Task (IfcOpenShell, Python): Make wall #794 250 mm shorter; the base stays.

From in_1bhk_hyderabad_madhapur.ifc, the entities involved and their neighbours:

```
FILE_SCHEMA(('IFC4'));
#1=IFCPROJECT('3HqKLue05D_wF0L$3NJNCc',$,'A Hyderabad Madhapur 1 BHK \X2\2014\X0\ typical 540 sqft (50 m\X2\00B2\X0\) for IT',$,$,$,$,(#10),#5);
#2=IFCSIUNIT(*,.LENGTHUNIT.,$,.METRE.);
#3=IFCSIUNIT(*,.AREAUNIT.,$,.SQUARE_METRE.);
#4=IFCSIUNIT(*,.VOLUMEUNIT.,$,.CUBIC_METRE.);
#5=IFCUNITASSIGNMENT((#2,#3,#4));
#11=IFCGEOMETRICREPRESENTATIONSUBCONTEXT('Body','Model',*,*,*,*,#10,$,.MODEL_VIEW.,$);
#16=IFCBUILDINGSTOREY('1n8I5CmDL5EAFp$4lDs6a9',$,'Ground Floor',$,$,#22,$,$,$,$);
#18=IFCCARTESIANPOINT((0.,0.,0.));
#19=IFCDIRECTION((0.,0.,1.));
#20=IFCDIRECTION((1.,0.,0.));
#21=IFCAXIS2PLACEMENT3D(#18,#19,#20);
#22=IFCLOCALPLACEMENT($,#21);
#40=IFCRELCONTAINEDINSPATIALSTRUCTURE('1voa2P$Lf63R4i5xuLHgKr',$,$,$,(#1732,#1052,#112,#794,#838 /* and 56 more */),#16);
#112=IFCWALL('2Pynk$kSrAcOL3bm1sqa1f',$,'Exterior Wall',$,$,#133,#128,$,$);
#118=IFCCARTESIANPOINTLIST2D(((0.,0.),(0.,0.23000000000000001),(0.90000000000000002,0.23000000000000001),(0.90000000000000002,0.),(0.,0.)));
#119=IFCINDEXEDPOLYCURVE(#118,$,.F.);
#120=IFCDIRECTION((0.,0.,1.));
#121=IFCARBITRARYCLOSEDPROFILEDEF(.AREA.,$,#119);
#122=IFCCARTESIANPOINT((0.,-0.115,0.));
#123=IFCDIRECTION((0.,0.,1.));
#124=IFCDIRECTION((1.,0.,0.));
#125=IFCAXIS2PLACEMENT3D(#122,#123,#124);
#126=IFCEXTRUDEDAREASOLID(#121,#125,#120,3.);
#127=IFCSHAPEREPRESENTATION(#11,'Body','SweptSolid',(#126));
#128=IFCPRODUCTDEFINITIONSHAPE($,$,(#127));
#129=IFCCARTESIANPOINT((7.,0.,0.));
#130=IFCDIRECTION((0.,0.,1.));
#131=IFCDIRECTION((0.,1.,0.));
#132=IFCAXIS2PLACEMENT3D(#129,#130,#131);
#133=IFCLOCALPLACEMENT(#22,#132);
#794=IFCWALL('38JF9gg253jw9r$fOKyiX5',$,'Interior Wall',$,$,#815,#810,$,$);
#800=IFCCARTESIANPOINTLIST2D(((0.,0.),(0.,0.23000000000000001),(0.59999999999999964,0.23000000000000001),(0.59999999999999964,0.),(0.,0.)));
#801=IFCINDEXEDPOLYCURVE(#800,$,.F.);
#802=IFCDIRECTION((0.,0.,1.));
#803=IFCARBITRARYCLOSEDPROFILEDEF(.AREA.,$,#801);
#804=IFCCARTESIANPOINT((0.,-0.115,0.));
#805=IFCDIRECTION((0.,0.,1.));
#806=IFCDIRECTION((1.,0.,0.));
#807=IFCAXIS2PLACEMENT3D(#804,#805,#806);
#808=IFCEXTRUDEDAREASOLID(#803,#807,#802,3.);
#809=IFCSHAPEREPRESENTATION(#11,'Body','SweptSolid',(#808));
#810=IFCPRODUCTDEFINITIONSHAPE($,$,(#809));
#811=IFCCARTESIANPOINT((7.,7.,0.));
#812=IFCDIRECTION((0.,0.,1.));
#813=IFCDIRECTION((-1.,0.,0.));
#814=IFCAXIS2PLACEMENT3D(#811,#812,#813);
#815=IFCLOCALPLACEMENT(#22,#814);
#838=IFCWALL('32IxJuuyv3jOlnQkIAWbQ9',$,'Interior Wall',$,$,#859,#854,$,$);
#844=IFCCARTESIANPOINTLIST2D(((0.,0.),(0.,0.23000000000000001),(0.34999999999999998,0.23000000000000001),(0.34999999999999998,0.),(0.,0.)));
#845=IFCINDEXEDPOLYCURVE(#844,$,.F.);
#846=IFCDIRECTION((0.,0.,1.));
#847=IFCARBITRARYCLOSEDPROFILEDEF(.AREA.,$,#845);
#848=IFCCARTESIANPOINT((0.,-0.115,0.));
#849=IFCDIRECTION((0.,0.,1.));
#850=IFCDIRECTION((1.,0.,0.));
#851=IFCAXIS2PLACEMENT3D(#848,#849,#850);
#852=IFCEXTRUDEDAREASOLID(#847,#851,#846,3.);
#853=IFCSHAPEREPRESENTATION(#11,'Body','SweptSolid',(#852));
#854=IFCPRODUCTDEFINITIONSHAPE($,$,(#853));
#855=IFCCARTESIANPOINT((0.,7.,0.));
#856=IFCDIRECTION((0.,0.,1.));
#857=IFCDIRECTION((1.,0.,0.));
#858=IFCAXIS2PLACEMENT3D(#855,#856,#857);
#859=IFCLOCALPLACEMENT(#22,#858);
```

```python
import ifcopenshell
import ifcopenshell.geom
import ifcopenshell.util.representation
import ifcopenshell.util.shape

model = ifcopenshell.open("in_1bhk_hyderabad_madhapur.ifc")
settings = ifcopenshell.geom.settings()


def volume(element):
    """Net volume in cubic metres, openings subtracted."""
    shape = ifcopenshell.geom.create_shape(settings, element)
    return ifcopenshell.util.shape.get_volume(shape.geometry)


wall = model.by_guid("38JF9gg253jw9r$fOKyiX5")
before = volume(wall)

body = ifcopenshell.util.representation.get_representation(wall, "Model", "Body")
solid = body.Items[0]
old_height = solid.Depth
solid.Depth -= 0.25
after = volume(wall)

print(f"height {old_height:g} -> {solid.Depth:g}, volume {before:.3f} -> {after:.3f} m3")

model.write("in_1bhk_hyderabad_madhapur_edited.ifc")
```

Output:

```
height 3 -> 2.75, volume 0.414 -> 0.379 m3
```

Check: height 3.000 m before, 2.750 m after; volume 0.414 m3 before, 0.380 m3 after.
